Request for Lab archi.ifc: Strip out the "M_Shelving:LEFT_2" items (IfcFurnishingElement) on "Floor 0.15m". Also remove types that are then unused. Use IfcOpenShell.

First a look at what the model holds.

```python
import ifcopenshell
import ifcopenshell.util.element

model = ifcopenshell.open("Lab archi.ifc")
print(model.schema)
storey = next(s for s in model.by_type("IfcBuildingStorey") if s.Name == "Floor 0.15m")
furniture = [e for e in ifcopenshell.util.element.get_decomposition(storey) if e.is_a("IfcFurnishingElement")]
seen = {}
for e in furniture:
    element_type = ifcopenshell.util.element.get_type(e)
    name = element_type.Name if element_type not in (None, e) else None
    seen[name] = seen.get(name, 0) + 1
for name, count in sorted(seen.items(), key=str):
    print(count, "x", name)
```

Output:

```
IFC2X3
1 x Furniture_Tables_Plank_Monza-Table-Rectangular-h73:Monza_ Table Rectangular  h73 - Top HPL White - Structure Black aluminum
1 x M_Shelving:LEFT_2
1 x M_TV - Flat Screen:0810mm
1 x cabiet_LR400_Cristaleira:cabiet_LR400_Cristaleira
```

```python
import ifcopenshell
import ifcopenshell.api.root
import ifcopenshell.util.element

model = ifcopenshell.open("Lab archi.ifc")

storey = next(s for s in model.by_type("IfcBuildingStorey") if s.Name == "Floor 0.15m")
furniture = [e for e in ifcopenshell.util.element.get_decomposition(storey) if e.is_a("IfcFurnishingElement")]
targets = [e for e in furniture if (t := ifcopenshell.util.element.get_type(e)) not in (None, e) and t.Name == "M_Shelving:LEFT_2"]
types = {ifcopenshell.util.element.get_type(e) for e in targets} - {None, *targets}

for e in targets:
    ifcopenshell.api.root.remove_product(model, product=e)
print(len(targets), "removed")

unused = [t for t in types if not ifcopenshell.util.element.get_types(t)]
for t in unused:
    ifcopenshell.api.root.remove_product(model, product=t)
print(len(unused), "unused types removed")

model.write("Lab archi_edited.ifc")
```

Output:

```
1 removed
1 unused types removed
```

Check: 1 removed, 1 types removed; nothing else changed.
